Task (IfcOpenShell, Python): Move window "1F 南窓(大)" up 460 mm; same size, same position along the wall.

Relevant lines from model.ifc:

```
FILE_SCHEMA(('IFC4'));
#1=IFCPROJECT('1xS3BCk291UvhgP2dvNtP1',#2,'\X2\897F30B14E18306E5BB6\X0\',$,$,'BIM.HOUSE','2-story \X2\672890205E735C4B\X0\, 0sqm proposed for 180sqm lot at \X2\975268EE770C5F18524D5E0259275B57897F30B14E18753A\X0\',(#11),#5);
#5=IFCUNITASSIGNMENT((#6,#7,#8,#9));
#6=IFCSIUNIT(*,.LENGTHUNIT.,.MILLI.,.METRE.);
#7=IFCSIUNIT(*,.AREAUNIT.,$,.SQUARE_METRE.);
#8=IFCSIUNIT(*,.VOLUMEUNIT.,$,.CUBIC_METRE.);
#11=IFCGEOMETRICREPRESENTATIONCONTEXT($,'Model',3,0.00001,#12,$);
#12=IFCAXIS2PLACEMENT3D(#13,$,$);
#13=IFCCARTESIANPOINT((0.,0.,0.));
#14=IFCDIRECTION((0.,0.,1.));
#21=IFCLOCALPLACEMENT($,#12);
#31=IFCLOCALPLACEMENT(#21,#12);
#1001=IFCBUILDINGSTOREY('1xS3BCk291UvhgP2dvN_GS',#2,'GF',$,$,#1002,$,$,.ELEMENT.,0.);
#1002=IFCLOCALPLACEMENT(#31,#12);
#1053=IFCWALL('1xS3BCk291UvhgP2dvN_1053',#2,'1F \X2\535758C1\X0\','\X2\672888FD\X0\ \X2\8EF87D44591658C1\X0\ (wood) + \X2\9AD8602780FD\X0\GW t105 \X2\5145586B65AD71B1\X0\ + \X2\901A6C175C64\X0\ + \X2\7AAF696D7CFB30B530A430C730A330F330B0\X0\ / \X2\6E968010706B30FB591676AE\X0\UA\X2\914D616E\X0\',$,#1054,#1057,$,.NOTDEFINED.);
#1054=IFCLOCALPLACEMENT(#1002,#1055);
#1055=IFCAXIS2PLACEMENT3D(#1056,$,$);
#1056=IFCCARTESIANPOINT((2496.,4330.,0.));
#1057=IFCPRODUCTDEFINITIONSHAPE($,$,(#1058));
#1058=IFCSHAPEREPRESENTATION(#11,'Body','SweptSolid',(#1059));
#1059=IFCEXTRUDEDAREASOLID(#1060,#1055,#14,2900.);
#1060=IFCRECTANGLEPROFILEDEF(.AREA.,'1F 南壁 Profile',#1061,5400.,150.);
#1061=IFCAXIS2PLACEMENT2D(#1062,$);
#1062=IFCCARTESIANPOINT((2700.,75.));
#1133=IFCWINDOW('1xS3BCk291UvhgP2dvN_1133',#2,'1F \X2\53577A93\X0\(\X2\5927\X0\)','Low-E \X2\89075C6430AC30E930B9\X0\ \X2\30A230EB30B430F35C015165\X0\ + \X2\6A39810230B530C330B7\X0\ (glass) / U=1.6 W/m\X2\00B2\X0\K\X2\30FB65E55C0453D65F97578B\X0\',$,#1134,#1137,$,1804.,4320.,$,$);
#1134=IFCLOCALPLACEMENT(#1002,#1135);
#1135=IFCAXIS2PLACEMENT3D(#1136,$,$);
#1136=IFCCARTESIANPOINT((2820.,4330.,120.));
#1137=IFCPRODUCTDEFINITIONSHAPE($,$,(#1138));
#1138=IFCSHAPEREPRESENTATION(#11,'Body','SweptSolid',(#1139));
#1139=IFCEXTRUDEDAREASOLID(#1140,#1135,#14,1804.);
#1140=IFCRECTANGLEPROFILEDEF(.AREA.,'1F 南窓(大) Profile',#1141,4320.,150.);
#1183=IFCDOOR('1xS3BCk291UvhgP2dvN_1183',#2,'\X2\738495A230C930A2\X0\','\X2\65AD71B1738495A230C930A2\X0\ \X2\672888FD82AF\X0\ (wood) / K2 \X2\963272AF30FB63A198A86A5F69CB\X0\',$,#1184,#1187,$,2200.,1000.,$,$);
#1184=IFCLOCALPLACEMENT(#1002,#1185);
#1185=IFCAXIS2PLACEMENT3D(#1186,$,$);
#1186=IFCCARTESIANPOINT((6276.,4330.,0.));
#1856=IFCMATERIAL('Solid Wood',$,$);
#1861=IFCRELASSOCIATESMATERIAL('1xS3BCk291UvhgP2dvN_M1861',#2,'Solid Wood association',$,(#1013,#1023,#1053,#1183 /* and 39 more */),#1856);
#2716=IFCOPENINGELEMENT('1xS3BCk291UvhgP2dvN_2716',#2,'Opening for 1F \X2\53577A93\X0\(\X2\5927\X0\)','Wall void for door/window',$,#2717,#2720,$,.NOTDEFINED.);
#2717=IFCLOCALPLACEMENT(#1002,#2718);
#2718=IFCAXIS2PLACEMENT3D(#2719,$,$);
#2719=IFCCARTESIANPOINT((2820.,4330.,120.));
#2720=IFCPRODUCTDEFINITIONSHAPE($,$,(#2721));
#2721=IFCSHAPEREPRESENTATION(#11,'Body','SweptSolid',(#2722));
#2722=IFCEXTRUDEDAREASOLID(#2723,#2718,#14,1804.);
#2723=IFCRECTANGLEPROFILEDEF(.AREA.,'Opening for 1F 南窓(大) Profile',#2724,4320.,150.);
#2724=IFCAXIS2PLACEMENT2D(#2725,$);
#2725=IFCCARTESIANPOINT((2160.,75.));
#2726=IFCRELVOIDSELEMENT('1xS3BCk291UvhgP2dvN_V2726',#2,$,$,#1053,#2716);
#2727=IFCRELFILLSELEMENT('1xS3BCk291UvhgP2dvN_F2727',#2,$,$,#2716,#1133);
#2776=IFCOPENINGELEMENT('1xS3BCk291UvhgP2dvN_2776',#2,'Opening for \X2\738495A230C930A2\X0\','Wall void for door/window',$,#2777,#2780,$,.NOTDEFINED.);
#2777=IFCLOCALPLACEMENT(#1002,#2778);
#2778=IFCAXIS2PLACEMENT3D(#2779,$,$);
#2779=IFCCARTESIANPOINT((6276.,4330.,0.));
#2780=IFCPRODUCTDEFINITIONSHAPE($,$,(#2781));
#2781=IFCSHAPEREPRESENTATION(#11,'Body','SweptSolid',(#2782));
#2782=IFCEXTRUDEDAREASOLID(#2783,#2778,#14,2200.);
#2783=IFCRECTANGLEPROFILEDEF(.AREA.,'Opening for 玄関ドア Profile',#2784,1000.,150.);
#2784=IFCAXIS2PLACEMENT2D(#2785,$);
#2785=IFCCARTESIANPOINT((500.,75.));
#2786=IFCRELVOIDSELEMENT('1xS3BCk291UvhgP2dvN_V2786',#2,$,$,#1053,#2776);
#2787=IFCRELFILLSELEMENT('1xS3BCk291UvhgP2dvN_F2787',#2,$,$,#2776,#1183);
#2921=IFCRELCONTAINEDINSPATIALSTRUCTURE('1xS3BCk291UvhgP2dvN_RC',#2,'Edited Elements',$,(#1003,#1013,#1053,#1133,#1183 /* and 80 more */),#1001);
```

```python
import numpy as np
import ifcopenshell
import ifcopenshell.api.geometry
import ifcopenshell.util.placement
import ifcopenshell.util.unit

model = ifcopenshell.open("model.ifc")
unit_scale = ifcopenshell.util.unit.calculate_unit_scale(model)

window = model.by_guid("1xS3BCk291UvhgP2dvN_1133")
opening = window.FillsVoids[0].RelatingOpeningElement
dz = 0.46 / unit_scale

shift = np.array([0.0, 0.0, dz])
# The window is not placed relative to its opening, so move both.
for product in (opening, window):
    matrix = ifcopenshell.util.placement.get_local_placement(product.ObjectPlacement)
    matrix[:3, 3] += shift
    ifcopenshell.api.geometry.edit_object_placement(model, product=product, matrix=matrix, is_si=False)

print(f"moved by {dz * unit_scale:+.3f} m")

model.write("model-out.ifc")
```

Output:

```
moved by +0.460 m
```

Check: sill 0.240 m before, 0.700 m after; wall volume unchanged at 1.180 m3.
